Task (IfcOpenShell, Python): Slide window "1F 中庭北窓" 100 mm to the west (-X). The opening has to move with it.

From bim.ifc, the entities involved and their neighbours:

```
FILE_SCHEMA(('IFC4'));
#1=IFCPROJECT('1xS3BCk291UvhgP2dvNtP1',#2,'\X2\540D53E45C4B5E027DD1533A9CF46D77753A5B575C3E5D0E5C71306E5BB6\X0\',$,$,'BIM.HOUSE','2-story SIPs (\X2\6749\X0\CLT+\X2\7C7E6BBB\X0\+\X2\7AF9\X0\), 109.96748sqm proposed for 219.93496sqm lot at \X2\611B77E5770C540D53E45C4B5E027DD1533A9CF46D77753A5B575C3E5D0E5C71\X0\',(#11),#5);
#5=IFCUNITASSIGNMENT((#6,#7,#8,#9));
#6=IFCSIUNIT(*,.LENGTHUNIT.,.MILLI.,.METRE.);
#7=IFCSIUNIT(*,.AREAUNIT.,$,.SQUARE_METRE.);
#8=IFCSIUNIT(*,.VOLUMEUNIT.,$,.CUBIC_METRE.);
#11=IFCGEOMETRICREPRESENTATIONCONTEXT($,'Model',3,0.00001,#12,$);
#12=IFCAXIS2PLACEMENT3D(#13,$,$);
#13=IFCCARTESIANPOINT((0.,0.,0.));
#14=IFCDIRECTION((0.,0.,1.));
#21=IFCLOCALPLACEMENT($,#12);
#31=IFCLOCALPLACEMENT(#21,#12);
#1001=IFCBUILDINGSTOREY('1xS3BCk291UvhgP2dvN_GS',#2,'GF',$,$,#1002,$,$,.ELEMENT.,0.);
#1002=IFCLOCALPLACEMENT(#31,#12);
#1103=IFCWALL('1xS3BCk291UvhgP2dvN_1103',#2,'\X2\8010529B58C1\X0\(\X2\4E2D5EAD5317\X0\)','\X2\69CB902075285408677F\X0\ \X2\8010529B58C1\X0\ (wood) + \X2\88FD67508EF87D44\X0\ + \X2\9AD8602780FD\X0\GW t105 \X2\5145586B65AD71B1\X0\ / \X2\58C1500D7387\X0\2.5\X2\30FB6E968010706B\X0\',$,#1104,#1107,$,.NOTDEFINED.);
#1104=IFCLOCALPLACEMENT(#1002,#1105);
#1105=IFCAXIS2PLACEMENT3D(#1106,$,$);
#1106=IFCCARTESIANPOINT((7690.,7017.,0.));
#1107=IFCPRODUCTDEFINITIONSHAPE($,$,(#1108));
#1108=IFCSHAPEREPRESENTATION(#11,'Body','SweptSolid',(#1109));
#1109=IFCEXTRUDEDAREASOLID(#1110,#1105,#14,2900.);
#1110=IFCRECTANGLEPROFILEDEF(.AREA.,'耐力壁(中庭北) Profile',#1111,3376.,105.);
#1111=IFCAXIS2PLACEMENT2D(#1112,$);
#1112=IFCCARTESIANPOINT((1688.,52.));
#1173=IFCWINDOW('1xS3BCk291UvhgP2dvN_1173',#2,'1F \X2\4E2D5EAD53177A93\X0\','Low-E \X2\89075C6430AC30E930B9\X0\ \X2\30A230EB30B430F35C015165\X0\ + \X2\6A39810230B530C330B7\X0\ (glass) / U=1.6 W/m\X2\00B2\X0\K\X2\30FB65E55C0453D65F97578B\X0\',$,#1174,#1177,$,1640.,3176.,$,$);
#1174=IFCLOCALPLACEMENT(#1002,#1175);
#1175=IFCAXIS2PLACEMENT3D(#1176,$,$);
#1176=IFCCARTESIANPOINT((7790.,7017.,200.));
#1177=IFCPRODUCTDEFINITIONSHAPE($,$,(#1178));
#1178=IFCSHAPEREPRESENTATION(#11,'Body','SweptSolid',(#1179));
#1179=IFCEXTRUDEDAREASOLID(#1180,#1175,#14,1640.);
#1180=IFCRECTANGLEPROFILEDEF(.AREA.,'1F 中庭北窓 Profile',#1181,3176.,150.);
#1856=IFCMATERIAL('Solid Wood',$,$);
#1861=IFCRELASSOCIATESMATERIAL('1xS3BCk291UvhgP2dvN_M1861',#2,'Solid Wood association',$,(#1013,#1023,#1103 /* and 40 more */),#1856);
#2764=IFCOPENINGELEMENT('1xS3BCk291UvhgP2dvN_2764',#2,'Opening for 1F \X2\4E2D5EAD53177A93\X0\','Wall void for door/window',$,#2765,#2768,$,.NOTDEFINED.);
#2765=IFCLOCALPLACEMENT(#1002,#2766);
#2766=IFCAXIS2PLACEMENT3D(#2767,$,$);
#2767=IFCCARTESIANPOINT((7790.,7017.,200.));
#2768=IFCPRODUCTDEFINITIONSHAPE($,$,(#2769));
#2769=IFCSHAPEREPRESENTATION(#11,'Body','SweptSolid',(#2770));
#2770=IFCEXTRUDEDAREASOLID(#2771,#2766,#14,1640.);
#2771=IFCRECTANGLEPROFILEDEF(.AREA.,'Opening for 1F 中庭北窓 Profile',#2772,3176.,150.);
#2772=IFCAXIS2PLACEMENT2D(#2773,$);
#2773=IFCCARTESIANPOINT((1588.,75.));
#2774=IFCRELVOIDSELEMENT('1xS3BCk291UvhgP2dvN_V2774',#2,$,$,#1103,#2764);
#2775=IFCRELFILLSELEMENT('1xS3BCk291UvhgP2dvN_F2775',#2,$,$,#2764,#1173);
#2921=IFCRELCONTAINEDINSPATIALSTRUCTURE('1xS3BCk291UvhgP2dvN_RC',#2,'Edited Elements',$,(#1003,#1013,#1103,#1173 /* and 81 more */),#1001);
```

```python
import ifcopenshell
import ifcopenshell.api.geometry
import ifcopenshell.util.placement
import ifcopenshell.util.unit

model = ifcopenshell.open("bim.ifc")
unit_scale = ifcopenshell.util.unit.calculate_unit_scale(model)

window = model.by_guid("1xS3BCk291UvhgP2dvN_1173")
opening = window.FillsVoids[0].RelatingOpeningElement
wall = opening.VoidsElements[0].RelatingBuildingElement

wall_matrix = ifcopenshell.util.placement.get_local_placement(wall.ObjectPlacement)
shift = wall_matrix[:3, 0] * -0.1 / unit_scale
before = ifcopenshell.util.placement.get_local_placement(window.ObjectPlacement)[:3, 3].copy()

# The window is not placed relative to its opening, so move both.
for product in (opening, window):
    matrix = ifcopenshell.util.placement.get_local_placement(product.ObjectPlacement)
    matrix[:3, 3] += shift
    ifcopenshell.api.geometry.edit_object_placement(model, product=product, matrix=matrix, is_si=False)

after = ifcopenshell.util.placement.get_local_placement(window.ObjectPlacement)[:3, 3]
print("window moved by", (after - before).round(3) + 0.0)

model.write("bim_rev.ifc")
```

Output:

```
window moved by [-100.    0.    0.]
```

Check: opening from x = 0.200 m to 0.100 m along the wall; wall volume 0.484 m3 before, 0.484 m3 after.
